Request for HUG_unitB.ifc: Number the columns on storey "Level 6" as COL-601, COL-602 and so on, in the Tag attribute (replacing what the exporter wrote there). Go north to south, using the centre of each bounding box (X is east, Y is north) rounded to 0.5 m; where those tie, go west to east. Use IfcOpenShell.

First a look at what the model holds.

```python
import ifcopenshell
import ifcopenshell.util.element
import ifcopenshell.util.placement

model = ifcopenshell.open("HUG_unitB.ifc")
print(model.schema)
storey = next(s for s in model.by_type("IfcBuildingStorey") if s.Name == "Level 6")
columns = [e for e in ifcopenshell.util.element.get_decomposition(storey) if e.is_a("IfcColumn")]
for e in sorted(columns, key=lambda e: e.id()):
    origin = ifcopenshell.util.placement.get_local_placement(e.ObjectPlacement)[:3, 3]
    print(e.id(), e.Tag, e.Name, origin.round(2) + 0.0, sep=" | ")
```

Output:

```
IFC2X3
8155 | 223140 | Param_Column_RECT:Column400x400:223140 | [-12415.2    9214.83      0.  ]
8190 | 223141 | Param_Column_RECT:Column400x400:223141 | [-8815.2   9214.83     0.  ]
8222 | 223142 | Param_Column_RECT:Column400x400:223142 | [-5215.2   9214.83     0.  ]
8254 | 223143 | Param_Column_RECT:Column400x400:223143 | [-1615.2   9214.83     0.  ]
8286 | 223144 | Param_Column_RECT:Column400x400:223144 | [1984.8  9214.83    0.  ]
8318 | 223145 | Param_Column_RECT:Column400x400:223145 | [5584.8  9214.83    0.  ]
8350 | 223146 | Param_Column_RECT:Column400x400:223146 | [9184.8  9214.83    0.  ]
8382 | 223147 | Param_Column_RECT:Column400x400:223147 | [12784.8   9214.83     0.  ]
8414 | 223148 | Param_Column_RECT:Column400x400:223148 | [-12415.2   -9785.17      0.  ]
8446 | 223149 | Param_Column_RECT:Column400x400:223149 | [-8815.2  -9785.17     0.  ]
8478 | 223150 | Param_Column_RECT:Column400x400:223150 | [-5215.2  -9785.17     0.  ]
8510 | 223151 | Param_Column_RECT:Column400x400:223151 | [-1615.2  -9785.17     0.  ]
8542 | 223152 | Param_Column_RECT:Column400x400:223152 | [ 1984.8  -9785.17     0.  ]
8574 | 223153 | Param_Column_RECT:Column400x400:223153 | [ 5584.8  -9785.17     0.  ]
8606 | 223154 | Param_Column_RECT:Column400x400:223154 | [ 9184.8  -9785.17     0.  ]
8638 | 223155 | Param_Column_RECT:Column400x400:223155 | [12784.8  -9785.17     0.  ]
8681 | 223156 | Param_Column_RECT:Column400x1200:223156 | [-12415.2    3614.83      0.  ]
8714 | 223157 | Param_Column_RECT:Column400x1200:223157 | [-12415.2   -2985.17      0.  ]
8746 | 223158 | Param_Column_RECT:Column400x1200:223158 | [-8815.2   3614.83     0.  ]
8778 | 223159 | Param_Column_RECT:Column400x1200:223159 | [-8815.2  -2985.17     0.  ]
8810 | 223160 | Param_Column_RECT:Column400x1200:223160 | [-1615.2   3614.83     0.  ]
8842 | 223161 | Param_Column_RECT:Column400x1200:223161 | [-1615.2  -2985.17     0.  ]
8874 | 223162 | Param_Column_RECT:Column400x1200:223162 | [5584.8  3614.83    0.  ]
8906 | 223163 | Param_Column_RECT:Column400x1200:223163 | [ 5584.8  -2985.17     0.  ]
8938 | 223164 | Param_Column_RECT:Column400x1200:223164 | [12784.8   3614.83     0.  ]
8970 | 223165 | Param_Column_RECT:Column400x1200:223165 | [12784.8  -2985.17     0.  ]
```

```python
import ifcopenshell
import ifcopenshell.geom
import ifcopenshell.util.element
import ifcopenshell.util.shape

model = ifcopenshell.open("HUG_unitB.ifc")
settings = ifcopenshell.geom.settings()
settings.set("use-world-coords", True)


def centre(element):
    shape = ifcopenshell.geom.create_shape(settings, element)
    return ifcopenshell.util.shape.get_bbox_centroid(shape.geometry)


storey = next(s for s in model.by_type("IfcBuildingStorey") if s.Name == "Level 6")
columns = [e for e in ifcopenshell.util.element.get_decomposition(storey) if e.is_a("IfcColumn")]

# Insertion points can sit at a corner or the storey origin, so sort by the geometry (in metres).
centres = {e: centre(e) for e in columns}
columns.sort(key=lambda e: (-round(centres[e][1] / 0.5), centres[e][0]))

for i, e in enumerate(columns, start=1):
    number = f"COL-6{i:02d}"
    e.Tag = number
    print(e.id(), number)

model.write("HUG_unitB_v2.ifc")
```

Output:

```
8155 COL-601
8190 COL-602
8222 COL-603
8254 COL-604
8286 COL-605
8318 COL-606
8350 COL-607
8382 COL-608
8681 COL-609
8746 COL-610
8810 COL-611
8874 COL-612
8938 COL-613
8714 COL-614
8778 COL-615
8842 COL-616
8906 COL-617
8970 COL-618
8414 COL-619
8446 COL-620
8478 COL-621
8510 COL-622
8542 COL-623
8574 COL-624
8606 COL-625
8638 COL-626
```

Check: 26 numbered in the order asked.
